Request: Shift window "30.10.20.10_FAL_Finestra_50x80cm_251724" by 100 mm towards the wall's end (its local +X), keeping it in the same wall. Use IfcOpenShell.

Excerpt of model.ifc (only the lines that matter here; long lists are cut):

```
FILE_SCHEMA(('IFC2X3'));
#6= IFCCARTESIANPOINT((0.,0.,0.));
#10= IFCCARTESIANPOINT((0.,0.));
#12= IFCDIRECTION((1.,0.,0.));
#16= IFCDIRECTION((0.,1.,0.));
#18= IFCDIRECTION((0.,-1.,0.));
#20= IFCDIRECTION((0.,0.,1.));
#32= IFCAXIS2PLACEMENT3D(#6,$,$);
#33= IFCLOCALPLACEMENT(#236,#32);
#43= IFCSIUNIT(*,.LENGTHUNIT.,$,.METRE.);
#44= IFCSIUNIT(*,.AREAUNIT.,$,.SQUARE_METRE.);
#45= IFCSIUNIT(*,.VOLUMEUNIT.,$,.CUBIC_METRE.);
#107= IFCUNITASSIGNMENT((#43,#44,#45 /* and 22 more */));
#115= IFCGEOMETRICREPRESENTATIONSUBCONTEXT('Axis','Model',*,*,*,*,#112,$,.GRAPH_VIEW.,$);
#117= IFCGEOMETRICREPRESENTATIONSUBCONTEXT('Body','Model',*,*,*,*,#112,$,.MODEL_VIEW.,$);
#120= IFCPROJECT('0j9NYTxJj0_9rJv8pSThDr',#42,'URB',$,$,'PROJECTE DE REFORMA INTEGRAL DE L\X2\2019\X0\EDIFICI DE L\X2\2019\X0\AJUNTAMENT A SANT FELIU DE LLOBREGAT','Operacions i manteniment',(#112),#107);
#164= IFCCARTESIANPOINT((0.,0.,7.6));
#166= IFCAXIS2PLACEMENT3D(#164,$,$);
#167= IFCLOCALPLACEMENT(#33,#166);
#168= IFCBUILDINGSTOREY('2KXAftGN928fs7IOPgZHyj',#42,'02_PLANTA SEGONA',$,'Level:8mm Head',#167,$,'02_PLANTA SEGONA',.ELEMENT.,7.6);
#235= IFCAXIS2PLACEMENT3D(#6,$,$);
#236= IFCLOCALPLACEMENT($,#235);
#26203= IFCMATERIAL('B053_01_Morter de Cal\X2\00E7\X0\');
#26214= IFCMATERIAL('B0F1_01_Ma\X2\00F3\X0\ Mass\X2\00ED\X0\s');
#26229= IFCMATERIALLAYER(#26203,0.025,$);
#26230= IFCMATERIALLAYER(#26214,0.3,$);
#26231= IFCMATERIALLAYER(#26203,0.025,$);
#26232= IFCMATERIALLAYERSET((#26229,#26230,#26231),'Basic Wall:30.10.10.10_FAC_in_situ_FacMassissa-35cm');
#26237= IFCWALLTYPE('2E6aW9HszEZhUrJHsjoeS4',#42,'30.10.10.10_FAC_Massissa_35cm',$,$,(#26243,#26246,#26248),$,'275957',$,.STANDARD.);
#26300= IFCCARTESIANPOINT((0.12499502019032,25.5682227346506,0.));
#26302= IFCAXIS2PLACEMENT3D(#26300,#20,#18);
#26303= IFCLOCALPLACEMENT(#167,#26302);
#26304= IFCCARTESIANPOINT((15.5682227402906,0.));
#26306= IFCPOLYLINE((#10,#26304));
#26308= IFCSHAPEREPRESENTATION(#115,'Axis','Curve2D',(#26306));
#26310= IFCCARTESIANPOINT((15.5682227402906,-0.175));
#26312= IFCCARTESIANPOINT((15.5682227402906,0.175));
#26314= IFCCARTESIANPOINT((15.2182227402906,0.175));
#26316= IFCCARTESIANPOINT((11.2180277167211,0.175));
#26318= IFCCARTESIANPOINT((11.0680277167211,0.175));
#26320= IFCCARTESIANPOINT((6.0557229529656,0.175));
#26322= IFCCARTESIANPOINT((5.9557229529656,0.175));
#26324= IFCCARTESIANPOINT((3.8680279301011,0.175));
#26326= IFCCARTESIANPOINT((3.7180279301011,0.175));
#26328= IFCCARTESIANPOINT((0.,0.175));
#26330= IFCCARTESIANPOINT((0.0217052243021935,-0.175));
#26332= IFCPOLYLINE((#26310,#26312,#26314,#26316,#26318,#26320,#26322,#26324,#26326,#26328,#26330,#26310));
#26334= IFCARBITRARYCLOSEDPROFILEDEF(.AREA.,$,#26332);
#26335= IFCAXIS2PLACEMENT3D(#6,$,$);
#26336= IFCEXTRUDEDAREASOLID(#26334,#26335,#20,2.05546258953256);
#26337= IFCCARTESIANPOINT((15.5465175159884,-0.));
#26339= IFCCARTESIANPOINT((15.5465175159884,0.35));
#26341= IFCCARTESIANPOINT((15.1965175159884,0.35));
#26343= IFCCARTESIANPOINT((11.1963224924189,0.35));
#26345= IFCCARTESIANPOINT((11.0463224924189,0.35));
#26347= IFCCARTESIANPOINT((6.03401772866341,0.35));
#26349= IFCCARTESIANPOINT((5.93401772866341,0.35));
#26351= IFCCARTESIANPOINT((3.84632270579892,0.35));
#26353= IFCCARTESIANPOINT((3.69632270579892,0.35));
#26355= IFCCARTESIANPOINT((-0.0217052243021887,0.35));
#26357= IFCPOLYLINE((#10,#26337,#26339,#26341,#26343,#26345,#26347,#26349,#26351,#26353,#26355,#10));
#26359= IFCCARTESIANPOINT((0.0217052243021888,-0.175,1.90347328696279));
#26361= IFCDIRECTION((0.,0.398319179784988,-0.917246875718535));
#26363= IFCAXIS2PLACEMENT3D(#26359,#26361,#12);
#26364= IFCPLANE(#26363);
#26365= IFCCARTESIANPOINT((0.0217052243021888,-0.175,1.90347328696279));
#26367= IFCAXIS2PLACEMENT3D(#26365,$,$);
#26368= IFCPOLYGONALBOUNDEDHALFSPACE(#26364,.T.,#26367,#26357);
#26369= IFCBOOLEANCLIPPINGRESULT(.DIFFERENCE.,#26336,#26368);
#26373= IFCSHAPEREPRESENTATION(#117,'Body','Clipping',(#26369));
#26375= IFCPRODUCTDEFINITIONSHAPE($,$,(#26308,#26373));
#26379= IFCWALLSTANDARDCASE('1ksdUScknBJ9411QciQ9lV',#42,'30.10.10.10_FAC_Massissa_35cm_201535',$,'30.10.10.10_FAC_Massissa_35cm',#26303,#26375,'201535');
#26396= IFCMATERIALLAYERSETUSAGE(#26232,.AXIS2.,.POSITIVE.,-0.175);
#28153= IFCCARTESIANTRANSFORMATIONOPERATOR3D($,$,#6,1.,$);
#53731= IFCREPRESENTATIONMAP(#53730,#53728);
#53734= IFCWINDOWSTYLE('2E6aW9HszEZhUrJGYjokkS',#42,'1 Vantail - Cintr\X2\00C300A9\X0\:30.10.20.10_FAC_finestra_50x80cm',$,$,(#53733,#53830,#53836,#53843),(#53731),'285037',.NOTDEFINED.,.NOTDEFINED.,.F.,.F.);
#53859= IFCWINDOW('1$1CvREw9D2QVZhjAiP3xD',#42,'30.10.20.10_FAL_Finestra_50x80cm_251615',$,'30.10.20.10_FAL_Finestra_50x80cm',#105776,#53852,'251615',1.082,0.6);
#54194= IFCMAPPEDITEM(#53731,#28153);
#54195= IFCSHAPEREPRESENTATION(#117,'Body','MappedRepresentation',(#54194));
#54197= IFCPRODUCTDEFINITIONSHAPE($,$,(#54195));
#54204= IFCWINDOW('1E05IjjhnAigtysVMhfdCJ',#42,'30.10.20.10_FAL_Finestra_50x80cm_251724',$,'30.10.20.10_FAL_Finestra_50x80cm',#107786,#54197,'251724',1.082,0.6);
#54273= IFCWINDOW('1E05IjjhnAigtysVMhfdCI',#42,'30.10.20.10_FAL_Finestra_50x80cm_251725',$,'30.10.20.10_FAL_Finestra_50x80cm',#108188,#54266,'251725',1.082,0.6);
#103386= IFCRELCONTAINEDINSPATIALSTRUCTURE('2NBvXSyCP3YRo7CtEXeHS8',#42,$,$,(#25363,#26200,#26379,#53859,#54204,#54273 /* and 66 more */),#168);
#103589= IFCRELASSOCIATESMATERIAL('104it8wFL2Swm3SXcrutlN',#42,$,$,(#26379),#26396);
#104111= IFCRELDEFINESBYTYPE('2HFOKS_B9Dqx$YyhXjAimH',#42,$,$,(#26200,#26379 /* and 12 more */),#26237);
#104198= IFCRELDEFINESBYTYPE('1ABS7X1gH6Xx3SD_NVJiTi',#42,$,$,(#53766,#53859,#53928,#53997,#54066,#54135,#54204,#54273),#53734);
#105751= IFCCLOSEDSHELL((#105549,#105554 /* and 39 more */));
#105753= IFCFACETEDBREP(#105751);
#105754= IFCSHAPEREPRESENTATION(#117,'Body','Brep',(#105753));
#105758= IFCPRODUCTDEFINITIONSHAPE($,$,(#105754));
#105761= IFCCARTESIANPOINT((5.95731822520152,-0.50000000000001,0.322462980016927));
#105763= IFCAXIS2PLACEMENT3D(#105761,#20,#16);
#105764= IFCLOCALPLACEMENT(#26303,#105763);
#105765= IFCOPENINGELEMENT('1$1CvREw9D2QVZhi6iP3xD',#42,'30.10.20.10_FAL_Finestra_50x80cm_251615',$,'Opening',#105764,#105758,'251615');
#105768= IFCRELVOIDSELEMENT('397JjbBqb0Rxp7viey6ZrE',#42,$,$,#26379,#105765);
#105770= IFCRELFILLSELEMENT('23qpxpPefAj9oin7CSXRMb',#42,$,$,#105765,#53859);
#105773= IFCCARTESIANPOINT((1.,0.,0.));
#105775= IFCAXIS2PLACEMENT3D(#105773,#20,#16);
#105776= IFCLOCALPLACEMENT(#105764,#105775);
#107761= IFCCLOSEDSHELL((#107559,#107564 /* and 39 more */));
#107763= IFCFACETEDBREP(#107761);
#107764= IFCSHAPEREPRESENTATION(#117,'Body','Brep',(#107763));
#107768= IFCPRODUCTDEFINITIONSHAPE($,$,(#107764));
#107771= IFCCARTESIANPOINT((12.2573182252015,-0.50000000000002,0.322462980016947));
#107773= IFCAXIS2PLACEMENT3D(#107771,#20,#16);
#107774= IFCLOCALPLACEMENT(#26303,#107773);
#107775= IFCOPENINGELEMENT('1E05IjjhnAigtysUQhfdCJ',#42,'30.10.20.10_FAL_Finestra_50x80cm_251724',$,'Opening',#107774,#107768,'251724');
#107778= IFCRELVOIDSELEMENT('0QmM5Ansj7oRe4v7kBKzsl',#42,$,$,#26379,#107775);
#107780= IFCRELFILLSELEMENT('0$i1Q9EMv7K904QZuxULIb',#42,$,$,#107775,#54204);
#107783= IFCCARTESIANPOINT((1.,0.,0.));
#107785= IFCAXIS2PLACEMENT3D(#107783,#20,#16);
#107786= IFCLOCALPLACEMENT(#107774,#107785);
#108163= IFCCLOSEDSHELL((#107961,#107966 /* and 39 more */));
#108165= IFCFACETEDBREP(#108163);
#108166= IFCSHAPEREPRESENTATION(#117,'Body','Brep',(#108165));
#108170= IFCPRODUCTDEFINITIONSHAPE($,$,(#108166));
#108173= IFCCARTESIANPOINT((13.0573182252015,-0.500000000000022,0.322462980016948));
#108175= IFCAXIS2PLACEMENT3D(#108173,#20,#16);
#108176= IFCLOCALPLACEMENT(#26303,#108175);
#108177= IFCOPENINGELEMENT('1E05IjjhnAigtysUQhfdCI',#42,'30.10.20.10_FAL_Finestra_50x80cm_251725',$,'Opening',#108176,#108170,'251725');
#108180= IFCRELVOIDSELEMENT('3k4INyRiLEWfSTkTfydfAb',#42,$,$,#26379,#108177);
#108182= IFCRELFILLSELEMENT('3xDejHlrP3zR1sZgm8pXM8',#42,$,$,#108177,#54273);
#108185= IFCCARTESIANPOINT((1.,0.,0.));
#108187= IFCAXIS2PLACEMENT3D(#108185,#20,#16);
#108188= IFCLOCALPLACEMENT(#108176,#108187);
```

```python
import ifcopenshell
import ifcopenshell.api.geometry
import ifcopenshell.util.placement
import ifcopenshell.util.unit

model = ifcopenshell.open("model.ifc")
unit_scale = ifcopenshell.util.unit.calculate_unit_scale(model)

window = model.by_guid("1E05IjjhnAigtysVMhfdCJ")
opening = window.FillsVoids[0].RelatingOpeningElement
wall = opening.VoidsElements[0].RelatingBuildingElement

wall_matrix = ifcopenshell.util.placement.get_local_placement(wall.ObjectPlacement)
shift = wall_matrix[:3, 0] * 0.1 / unit_scale
before = ifcopenshell.util.placement.get_local_placement(window.ObjectPlacement)[:3, 3].copy()

# The window is placed relative to its opening, so it follows when the opening moves.
matrix = ifcopenshell.util.placement.get_local_placement(opening.ObjectPlacement)
matrix[:3, 3] += shift
ifcopenshell.api.geometry.edit_object_placement(
    model, product=opening, matrix=matrix, is_si=False, should_transform_children=True
)

after = ifcopenshell.util.placement.get_local_placement(window.ObjectPlacement)[:3, 3]
print("window moved by", (after - before).round(3) + 0.0)

model.write("model_edited.ifc")
```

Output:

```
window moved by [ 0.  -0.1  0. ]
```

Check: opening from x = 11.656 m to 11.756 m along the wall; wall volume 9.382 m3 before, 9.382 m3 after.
